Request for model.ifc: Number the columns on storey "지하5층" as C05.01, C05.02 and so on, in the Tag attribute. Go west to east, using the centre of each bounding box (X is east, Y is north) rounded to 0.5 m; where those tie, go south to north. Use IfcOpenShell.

First a look at what the model holds.

```python
import ifcopenshell
import ifcopenshell.util.element
import ifcopenshell.util.placement

model = ifcopenshell.open("model.ifc")
print(model.schema)
storey = next(s for s in model.by_type("IfcBuildingStorey") if s.Name == "지하5층")
columns = [e for e in ifcopenshell.util.element.get_decomposition(storey) if e.is_a("IfcColumn")]
for e in sorted(columns, key=lambda e: e.id()):
    origin = ifcopenshell.util.placement.get_local_placement(e.ObjectPlacement)[:3, 3]
    print(e.id(), e.Tag, e.Name, origin.round(2) + 0.0, sep=" | ")
```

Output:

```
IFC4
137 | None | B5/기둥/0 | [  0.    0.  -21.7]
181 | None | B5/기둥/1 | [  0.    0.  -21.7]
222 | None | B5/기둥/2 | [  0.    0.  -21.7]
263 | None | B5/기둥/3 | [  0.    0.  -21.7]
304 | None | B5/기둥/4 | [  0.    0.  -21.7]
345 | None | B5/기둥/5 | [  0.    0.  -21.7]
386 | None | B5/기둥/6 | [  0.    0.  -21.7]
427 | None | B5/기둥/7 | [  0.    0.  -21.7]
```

```python
import ifcopenshell
import ifcopenshell.geom
import ifcopenshell.util.element
import ifcopenshell.util.shape

model = ifcopenshell.open("model.ifc")
settings = ifcopenshell.geom.settings()
settings.set("use-world-coords", True)


def centre(element):
    shape = ifcopenshell.geom.create_shape(settings, element)
    return ifcopenshell.util.shape.get_bbox_centroid(shape.geometry)


storey = next(s for s in model.by_type("IfcBuildingStorey") if s.Name == "지하5층")
columns = [e for e in ifcopenshell.util.element.get_decomposition(storey) if e.is_a("IfcColumn")]

# Insertion points can sit at a corner or the storey origin, so sort by the geometry (in metres).
centres = {e: centre(e) for e in columns}
columns.sort(key=lambda e: (round(centres[e][0] / 0.5), centres[e][1]))

for i, e in enumerate(columns, start=1):
    number = f"C05.{i:02d}"
    e.Tag = number
    print(e.id(), number)

model.write("model_updated.ifc")
```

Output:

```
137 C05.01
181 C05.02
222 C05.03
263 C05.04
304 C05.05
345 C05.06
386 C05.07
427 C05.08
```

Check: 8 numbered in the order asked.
